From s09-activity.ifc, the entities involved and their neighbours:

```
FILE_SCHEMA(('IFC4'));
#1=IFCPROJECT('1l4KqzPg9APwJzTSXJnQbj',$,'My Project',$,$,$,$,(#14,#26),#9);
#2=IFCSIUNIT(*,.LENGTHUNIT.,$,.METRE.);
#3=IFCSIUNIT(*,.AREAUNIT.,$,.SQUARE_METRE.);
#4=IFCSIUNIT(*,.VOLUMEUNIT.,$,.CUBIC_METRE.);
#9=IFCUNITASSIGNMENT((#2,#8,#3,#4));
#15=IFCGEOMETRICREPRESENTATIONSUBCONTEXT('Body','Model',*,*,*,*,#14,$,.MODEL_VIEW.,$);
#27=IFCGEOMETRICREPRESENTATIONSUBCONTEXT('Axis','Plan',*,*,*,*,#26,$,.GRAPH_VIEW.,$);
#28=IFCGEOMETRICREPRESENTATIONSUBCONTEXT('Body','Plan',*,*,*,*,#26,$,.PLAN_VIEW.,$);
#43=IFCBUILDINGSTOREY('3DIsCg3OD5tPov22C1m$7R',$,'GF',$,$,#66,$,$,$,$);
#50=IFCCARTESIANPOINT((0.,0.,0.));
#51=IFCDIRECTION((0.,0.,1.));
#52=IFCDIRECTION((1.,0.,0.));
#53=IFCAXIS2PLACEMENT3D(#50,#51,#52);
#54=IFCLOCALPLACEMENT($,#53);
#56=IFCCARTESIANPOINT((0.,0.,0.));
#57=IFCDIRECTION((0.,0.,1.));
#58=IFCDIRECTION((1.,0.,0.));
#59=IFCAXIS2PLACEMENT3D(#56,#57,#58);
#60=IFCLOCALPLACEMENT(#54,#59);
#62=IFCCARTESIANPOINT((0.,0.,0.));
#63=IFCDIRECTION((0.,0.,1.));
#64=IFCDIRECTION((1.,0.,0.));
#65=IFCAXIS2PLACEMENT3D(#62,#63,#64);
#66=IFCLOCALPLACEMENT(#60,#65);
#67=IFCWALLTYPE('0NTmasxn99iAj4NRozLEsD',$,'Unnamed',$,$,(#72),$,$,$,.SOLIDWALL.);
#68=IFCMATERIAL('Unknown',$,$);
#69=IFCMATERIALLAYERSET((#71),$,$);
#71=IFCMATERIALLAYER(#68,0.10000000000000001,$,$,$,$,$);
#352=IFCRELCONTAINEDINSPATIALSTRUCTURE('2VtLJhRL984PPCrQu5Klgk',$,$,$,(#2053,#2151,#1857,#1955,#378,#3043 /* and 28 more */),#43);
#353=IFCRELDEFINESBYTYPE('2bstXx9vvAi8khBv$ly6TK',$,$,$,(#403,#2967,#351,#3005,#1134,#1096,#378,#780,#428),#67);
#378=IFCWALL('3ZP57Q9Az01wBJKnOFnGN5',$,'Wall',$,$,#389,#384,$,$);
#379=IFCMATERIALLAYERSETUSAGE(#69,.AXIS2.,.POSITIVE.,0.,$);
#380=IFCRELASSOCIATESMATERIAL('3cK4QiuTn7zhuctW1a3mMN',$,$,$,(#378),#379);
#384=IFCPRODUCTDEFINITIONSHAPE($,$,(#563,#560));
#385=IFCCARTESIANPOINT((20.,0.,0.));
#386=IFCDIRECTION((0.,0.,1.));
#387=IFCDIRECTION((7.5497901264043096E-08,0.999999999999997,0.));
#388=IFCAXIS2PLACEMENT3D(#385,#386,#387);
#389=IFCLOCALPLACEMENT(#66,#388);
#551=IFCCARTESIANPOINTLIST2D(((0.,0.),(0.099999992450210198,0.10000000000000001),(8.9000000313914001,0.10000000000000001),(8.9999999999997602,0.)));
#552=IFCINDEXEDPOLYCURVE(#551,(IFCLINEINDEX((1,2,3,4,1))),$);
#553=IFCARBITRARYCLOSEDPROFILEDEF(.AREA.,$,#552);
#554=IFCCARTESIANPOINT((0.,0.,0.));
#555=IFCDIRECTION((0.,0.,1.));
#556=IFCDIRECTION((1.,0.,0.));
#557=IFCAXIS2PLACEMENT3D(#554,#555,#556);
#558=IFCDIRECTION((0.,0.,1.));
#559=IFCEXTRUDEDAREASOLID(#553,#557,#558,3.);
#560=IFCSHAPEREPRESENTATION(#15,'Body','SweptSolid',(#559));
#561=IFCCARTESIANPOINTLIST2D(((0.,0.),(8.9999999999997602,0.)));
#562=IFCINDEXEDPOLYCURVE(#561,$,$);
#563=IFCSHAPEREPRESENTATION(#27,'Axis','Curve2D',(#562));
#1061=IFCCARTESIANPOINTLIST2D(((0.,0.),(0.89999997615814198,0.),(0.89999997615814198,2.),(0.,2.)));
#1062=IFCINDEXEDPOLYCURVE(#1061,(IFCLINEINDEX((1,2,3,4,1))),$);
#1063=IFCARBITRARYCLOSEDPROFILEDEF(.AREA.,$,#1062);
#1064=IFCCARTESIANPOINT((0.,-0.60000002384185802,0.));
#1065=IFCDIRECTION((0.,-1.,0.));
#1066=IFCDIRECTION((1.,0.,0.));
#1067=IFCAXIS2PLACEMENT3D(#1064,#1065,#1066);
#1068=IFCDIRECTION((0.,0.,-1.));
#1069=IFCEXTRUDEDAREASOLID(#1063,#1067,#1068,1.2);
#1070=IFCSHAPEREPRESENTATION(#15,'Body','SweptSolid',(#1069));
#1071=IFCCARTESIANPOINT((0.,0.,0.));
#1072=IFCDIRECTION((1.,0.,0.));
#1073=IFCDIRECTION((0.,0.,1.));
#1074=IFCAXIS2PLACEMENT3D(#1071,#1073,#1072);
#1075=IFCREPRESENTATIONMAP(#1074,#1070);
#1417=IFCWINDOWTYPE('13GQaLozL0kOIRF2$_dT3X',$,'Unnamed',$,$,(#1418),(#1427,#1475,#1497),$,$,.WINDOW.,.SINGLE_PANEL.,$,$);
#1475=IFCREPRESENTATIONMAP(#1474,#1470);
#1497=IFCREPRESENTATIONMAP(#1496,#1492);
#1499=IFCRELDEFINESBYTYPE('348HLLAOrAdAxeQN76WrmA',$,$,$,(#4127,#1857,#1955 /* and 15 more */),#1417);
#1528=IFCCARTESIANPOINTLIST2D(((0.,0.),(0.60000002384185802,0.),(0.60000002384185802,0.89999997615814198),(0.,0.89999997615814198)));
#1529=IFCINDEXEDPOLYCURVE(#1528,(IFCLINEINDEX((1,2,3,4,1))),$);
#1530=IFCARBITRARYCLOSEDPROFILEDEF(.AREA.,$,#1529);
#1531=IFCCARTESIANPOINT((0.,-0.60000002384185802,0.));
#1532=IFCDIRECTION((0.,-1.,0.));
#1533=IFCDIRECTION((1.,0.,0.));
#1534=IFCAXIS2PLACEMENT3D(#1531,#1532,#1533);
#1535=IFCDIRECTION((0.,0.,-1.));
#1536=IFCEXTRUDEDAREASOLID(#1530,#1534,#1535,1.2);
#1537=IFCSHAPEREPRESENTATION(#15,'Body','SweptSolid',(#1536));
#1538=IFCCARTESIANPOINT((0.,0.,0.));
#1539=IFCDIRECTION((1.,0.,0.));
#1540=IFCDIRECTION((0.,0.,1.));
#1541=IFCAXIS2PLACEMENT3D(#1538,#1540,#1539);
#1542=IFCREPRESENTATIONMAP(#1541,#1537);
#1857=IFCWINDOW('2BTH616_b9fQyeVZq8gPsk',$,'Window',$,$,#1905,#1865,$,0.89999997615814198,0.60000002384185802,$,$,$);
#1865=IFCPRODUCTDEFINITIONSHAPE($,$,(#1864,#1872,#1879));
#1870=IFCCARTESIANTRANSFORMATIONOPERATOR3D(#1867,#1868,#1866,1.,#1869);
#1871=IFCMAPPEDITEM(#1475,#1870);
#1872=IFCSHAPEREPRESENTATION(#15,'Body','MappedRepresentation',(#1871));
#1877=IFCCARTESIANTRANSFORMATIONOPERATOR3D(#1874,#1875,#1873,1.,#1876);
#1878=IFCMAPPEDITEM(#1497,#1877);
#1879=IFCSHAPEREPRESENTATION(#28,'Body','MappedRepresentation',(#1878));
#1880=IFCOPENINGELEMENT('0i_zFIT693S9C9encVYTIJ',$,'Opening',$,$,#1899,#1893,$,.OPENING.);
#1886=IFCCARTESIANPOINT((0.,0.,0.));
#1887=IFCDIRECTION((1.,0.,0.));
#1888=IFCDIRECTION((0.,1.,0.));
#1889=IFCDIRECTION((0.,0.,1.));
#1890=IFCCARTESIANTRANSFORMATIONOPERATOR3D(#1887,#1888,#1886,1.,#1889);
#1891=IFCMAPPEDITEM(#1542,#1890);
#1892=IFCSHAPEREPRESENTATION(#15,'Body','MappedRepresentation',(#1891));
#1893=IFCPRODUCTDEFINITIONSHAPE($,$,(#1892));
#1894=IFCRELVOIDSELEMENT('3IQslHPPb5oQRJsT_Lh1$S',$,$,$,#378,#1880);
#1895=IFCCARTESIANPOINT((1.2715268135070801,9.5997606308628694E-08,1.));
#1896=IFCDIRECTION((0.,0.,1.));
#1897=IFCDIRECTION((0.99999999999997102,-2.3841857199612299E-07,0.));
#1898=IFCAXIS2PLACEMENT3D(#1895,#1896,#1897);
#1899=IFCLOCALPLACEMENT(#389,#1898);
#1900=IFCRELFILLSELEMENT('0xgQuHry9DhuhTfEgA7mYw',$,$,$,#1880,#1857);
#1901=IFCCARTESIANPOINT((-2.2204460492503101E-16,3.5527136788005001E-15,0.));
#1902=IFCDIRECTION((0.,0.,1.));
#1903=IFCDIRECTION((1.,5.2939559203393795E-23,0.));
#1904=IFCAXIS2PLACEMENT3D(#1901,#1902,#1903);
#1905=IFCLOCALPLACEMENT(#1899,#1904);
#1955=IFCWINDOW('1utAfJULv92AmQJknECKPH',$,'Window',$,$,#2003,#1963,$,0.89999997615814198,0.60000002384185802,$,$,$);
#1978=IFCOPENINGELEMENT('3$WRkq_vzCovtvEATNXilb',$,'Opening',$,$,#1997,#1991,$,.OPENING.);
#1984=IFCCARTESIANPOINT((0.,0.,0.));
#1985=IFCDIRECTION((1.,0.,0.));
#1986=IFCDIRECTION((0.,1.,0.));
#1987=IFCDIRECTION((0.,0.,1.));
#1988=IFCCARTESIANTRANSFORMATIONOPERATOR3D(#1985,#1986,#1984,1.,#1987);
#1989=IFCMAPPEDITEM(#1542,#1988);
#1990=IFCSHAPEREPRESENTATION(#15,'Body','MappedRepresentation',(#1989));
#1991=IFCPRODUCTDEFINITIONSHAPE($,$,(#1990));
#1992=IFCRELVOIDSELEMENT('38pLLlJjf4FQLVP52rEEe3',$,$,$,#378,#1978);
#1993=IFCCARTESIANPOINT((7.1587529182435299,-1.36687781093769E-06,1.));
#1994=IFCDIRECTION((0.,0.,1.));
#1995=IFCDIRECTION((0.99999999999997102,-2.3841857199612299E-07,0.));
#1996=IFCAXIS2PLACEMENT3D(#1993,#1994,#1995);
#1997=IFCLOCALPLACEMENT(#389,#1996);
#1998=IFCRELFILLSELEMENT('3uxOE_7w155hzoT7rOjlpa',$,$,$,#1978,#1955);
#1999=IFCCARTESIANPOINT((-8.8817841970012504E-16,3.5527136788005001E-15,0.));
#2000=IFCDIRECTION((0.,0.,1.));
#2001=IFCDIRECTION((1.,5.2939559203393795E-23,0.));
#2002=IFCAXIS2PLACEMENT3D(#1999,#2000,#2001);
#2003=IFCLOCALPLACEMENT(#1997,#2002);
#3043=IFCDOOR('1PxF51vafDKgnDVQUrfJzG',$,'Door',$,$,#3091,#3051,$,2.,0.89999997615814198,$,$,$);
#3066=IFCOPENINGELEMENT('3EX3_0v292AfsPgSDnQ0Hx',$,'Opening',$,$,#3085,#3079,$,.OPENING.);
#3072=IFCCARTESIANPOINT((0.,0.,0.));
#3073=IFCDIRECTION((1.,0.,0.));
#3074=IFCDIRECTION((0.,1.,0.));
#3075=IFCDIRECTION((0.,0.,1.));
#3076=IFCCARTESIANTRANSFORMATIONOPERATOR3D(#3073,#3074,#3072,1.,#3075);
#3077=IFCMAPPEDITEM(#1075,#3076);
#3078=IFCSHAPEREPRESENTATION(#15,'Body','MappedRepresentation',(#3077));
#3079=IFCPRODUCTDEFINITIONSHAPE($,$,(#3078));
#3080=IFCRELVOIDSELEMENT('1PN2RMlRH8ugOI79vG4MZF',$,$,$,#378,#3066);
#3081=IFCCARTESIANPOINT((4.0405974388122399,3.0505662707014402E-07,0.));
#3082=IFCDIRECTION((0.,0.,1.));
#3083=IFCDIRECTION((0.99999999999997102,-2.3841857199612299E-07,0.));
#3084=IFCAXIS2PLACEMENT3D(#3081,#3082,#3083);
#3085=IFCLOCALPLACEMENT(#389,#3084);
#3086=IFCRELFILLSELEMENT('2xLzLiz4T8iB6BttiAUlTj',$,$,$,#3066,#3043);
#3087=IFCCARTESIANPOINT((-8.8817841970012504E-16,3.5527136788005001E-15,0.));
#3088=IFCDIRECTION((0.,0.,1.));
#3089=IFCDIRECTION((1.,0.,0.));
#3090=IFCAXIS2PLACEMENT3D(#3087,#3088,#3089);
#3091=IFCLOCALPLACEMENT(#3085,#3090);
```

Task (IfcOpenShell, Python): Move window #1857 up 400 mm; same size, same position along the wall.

```python
import numpy as np
import ifcopenshell
import ifcopenshell.api.geometry
import ifcopenshell.util.placement
import ifcopenshell.util.unit

model = ifcopenshell.open("s09-activity.ifc")
unit_scale = ifcopenshell.util.unit.calculate_unit_scale(model)

window = model.by_id(1857)
opening = window.FillsVoids[0].RelatingOpeningElement
dz = 0.4 / unit_scale

shift = np.array([0.0, 0.0, dz])
# The window is placed relative to its opening, so it follows when the opening moves.
matrix = ifcopenshell.util.placement.get_local_placement(opening.ObjectPlacement)
matrix[:3, 3] += shift
ifcopenshell.api.geometry.edit_object_placement(
    model, product=opening, matrix=matrix, is_si=False, should_transform_children=True
)

print(f"moved by {dz * unit_scale:+.3f} m")

model.write("s09-activity_updated.ifc")
```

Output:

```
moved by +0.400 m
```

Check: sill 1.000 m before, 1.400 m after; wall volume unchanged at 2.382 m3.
